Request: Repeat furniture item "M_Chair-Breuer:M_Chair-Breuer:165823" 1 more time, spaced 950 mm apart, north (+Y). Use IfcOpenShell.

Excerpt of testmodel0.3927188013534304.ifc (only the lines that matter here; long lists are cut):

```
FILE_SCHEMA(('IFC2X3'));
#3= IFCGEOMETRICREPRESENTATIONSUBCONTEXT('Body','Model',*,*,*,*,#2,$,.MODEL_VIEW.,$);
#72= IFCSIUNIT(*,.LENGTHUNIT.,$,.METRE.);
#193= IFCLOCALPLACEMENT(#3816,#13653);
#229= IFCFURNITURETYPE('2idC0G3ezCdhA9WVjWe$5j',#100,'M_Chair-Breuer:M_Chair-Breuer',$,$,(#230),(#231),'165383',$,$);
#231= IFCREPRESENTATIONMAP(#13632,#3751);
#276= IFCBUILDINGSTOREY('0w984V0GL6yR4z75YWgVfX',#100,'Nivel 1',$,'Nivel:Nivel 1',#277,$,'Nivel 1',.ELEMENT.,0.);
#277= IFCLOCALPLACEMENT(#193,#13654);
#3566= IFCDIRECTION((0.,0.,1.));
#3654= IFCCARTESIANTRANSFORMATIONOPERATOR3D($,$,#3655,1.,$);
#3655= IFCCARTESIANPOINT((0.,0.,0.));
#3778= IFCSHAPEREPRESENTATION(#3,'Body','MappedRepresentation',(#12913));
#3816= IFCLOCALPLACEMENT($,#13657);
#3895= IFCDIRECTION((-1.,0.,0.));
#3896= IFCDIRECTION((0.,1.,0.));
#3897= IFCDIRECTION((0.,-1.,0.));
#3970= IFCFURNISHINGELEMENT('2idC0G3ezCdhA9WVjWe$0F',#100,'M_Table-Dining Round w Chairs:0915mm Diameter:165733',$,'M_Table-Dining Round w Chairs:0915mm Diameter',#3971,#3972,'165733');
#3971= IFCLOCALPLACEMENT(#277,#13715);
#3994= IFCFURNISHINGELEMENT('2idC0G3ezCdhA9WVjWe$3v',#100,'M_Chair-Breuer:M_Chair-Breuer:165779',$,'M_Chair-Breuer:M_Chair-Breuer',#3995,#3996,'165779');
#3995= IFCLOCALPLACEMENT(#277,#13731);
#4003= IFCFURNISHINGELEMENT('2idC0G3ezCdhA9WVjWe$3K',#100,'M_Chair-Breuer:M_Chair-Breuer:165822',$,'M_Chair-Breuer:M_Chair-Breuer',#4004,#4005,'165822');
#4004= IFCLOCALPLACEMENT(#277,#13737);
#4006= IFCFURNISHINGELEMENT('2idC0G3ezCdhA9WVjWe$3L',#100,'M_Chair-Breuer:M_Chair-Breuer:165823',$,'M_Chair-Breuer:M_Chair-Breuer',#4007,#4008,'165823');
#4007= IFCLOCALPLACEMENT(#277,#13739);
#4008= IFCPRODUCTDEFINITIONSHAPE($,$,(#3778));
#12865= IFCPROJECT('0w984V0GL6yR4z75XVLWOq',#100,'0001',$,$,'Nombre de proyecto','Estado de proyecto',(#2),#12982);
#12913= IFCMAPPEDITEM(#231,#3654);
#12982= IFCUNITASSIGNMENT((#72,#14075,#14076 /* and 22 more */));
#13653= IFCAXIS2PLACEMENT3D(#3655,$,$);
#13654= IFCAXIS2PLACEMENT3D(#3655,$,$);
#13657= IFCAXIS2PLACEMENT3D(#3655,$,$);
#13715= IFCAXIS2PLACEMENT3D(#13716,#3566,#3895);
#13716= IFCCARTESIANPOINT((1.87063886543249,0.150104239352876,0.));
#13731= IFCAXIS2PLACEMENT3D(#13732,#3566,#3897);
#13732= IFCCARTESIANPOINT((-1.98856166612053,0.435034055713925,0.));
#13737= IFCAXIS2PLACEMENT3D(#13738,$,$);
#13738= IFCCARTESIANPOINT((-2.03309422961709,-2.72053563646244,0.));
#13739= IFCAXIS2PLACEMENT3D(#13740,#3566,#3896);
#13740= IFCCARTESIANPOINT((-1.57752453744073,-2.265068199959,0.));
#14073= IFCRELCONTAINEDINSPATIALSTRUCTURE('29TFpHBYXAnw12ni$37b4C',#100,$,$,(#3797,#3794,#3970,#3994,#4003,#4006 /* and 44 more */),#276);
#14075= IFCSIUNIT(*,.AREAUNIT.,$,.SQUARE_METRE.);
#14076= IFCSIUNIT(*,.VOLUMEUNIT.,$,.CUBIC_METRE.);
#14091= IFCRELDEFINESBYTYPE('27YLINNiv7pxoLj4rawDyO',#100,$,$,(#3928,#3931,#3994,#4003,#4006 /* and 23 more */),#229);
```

```python
import numpy as np
import ifcopenshell
import ifcopenshell.api.geometry
import ifcopenshell.api.root
import ifcopenshell.util.element
import ifcopenshell.util.placement

model = ifcopenshell.open("testmodel0.3927188013534304.ifc")


def reuse_history(source, copy):
    """copy_class also copies each property set's owner history, people and application; keep the originals."""
    for rel in copy.IsDefinedBy:
        if rel.is_a("IfcRelDefinesByProperties") and (history := rel.RelatingPropertyDefinition.OwnerHistory):
            rel.RelatingPropertyDefinition.OwnerHistory = source.OwnerHistory
            ifcopenshell.util.element.remove_deep2(model, history)


source = model.by_id(4006)
base = ifcopenshell.util.placement.get_local_placement(source.ObjectPlacement)
step = np.array([0.0, 1.0, 0.0]) * 0.95

for i in range(1, 2):
    copy = ifcopenshell.api.root.copy_class(model, product=source)
    copy.Representation = ifcopenshell.util.element.copy_deep(
        model, source.Representation, exclude=["IfcGeometricRepresentationContext", "IfcRepresentationMap"]
    )
    copy.Name = "M_Chair-Breuer:M_Chair-Breuer"
    copy.Tag = None
    reuse_history(source, copy)
    matrix = base.copy()
    matrix[:3, 3] += i * step
    print("added at", matrix[:3, 3].round(3) + 0.0)
    ifcopenshell.api.geometry.edit_object_placement(model, product=copy, matrix=matrix, is_si=False)

model.write("testmodel0.3927188013534304-out.ifc")
```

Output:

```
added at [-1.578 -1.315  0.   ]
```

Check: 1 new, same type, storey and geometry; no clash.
